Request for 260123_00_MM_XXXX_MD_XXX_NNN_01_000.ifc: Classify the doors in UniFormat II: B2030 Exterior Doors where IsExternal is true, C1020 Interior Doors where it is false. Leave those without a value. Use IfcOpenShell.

First a look at what the model holds.

```python
import ifcopenshell
import ifcopenshell.util.element

model = ifcopenshell.open("260123_00_MM_XXXX_MD_XXX_NNN_01_000.ifc")
print(model.schema)
print("classifications:", [c.Name for c in model.by_type("IfcClassification")])
values = [ifcopenshell.util.element.get_pset(e, "Pset_DoorCommon", "IsExternal") for e in model.by_type("IfcDoor")]
for value in (True, False, None):
    print("IsExternal", value, values.count(value))
```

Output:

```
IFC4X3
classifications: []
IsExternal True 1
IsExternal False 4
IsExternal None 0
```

```python
import ifcopenshell
import ifcopenshell.api.classification
import ifcopenshell.util.element

model = ifcopenshell.open("260123_00_MM_XXXX_MD_XXX_NNN_01_000.ifc")

system = ifcopenshell.api.classification.add_classification(model, classification="UniFormat II")

doors = model.by_type("IfcDoor")
external = {e: ifcopenshell.util.element.get_pset(e, "Pset_DoorCommon", "IsExternal") for e in doors}
for flag, code, name in ((True, "B2030", "Exterior Doors"), (False, "C1020", "Interior Doors")):
    products = [e for e in doors if external[e] is flag]
    ifcopenshell.api.classification.add_reference(
        model, products=products, classification=system, identification=code, name=name
    )
    print(code, len(products))

model.write("260123_00_MM_XXXX_MD_XXX_NNN_01_000_edited.ifc")
```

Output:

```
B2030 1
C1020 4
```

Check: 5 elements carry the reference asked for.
